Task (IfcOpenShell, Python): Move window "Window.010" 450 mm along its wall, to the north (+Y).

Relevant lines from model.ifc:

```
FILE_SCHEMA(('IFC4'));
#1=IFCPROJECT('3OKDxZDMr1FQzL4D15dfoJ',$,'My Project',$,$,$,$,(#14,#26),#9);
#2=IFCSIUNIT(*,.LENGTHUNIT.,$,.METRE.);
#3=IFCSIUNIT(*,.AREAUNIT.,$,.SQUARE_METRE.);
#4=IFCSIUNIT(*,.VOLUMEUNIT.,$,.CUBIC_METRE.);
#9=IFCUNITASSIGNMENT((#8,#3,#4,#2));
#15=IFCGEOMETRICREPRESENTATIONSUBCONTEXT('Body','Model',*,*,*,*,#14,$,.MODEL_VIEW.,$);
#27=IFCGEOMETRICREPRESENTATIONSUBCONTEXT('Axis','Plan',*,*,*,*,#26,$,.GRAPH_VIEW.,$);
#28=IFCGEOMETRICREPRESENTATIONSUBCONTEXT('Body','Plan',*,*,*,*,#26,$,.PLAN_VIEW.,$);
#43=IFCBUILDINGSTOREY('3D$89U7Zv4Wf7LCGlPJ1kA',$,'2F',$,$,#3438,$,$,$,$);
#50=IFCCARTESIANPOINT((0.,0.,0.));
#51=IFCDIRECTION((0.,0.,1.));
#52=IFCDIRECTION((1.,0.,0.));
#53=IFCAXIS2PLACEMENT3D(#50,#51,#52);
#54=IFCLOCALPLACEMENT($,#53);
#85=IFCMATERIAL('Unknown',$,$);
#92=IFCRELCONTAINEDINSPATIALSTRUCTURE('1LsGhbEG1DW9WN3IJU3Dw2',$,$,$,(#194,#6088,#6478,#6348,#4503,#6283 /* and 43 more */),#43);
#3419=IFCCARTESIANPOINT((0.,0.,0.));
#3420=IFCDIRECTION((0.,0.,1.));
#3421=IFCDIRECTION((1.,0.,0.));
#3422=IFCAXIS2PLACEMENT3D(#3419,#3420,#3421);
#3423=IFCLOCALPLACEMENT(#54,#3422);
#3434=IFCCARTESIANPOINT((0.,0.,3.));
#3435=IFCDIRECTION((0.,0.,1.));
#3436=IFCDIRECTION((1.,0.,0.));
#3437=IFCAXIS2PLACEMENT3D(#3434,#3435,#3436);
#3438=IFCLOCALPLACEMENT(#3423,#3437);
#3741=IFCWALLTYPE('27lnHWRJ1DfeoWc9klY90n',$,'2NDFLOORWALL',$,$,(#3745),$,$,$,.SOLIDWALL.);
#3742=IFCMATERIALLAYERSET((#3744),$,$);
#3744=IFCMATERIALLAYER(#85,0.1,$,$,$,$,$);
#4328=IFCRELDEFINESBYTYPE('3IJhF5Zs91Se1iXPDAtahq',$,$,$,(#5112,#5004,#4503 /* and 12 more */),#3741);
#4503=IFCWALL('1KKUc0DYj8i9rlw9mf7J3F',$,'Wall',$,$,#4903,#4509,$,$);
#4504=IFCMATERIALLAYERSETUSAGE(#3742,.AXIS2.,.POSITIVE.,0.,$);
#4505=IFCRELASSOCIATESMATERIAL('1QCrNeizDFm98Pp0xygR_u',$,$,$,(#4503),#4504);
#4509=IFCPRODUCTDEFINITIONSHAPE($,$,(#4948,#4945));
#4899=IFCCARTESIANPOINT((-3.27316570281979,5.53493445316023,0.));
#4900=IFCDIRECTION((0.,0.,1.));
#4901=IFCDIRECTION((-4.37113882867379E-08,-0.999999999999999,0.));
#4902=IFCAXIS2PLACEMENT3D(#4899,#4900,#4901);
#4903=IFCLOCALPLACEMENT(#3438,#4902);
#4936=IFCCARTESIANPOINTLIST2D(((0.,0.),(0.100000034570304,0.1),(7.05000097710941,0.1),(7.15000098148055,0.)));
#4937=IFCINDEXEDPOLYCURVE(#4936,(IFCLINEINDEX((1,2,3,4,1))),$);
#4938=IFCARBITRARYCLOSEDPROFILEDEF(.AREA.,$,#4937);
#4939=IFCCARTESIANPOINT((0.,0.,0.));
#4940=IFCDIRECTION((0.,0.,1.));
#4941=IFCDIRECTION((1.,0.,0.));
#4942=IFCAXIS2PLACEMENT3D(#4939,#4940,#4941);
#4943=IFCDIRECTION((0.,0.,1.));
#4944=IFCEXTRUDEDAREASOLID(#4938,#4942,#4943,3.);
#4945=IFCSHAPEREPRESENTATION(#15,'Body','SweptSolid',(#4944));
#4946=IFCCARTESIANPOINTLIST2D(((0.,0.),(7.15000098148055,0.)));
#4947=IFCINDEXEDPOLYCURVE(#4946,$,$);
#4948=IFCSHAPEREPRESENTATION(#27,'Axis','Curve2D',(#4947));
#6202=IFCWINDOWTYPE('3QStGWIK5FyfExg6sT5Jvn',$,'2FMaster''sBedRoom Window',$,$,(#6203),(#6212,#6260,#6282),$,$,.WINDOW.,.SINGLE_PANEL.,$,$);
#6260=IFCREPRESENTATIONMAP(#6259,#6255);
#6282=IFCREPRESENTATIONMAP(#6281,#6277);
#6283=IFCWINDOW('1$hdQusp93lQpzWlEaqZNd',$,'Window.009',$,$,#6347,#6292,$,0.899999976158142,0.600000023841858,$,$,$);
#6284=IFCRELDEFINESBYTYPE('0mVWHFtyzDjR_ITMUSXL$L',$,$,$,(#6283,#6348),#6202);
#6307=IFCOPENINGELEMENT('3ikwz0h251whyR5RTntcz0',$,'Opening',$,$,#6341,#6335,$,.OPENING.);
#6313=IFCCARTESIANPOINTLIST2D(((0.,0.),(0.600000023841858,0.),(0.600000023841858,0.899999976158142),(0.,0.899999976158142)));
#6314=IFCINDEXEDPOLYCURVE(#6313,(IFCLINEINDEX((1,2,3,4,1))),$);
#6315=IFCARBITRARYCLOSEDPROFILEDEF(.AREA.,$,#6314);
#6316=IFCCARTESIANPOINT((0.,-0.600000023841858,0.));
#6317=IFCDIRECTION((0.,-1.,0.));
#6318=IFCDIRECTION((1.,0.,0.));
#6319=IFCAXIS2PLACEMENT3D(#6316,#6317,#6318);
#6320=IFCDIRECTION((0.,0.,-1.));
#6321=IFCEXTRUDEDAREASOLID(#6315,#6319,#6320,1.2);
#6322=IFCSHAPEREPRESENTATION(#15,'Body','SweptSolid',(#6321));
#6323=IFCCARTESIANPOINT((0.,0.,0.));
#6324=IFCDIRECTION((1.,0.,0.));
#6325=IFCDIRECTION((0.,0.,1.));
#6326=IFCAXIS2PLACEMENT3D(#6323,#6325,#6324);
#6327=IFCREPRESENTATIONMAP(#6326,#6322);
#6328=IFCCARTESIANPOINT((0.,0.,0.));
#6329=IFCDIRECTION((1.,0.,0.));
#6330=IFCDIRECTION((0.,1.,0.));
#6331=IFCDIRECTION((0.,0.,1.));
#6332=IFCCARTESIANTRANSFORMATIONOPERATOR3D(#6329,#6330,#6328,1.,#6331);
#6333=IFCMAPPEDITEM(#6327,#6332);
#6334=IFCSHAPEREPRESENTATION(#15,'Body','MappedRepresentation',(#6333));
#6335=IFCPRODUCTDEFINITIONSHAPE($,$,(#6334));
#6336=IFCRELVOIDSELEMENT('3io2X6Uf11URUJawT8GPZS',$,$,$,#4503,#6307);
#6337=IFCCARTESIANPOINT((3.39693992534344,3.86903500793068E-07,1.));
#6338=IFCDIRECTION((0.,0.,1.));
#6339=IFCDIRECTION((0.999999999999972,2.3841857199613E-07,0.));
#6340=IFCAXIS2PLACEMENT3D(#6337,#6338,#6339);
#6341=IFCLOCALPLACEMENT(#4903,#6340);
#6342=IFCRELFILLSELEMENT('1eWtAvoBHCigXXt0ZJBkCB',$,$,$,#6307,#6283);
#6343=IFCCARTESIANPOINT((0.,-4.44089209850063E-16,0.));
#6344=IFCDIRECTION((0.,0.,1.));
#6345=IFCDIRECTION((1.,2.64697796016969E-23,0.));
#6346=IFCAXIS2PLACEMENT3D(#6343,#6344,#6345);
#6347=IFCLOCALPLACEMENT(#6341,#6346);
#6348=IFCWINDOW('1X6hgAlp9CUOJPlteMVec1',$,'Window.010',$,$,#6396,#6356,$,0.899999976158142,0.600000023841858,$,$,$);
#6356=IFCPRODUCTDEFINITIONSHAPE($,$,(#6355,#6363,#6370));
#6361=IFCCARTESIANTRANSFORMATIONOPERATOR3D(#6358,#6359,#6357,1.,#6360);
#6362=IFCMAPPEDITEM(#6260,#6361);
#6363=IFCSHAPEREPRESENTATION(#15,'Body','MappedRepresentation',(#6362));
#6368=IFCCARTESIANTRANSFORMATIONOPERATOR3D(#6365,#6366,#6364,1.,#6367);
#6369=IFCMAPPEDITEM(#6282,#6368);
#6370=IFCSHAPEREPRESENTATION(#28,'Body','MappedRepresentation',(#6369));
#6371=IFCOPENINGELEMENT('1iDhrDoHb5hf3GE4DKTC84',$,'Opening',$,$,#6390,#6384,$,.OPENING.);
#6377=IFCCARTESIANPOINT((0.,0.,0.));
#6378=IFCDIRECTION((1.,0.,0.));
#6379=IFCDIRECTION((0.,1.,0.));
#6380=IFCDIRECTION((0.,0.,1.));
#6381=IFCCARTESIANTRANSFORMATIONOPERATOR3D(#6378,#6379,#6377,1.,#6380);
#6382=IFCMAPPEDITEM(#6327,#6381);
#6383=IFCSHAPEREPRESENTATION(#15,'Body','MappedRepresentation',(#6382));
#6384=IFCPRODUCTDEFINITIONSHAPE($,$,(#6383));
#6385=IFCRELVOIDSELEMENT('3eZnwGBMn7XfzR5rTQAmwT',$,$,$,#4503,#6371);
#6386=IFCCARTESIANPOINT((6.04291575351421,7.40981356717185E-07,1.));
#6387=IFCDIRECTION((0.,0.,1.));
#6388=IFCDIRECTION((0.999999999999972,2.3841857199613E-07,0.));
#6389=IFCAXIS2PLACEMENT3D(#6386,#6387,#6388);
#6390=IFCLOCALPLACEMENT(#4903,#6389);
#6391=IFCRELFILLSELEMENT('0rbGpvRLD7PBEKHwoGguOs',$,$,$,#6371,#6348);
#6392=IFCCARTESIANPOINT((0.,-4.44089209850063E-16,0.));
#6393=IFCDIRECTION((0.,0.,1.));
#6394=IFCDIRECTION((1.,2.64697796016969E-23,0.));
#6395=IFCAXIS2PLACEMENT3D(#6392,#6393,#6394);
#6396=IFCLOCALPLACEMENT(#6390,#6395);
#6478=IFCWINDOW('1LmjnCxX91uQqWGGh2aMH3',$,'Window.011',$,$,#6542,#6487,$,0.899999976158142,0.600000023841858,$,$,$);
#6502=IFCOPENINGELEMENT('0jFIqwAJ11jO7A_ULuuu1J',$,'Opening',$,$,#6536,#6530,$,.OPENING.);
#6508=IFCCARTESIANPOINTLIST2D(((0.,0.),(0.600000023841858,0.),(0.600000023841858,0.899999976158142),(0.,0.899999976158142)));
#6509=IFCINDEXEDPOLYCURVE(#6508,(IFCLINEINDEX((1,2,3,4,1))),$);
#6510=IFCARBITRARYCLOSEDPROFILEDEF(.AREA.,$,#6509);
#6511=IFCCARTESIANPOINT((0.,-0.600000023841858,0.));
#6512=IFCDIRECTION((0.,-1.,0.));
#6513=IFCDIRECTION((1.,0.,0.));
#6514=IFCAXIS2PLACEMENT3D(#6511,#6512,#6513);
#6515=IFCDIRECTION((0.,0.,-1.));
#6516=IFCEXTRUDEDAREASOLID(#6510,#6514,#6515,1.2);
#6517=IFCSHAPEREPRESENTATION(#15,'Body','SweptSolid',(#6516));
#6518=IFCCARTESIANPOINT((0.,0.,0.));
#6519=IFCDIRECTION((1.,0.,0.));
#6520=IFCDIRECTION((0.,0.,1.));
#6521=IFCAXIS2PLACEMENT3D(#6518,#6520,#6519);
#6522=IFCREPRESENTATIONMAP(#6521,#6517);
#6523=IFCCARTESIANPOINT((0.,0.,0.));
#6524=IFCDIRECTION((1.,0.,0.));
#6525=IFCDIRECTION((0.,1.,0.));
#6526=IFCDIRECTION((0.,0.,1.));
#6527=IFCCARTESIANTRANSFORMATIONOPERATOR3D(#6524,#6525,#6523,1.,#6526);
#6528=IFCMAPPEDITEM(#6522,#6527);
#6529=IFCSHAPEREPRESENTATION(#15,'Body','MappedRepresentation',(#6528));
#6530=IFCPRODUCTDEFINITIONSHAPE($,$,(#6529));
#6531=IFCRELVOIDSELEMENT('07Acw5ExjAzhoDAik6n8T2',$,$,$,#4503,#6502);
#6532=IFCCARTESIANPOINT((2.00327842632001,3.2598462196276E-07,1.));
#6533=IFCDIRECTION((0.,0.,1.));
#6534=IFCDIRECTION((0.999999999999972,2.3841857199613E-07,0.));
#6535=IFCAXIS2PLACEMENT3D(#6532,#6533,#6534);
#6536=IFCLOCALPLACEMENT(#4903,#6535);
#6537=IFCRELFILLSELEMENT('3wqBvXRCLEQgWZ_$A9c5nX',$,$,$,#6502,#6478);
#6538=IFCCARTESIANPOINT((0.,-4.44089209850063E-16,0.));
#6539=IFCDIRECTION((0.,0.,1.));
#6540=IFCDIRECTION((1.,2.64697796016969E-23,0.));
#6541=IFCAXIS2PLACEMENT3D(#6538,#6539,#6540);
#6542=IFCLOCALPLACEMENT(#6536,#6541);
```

```python
import ifcopenshell
import ifcopenshell.api.geometry
import ifcopenshell.util.placement
import ifcopenshell.util.unit

model = ifcopenshell.open("model.ifc")
unit_scale = ifcopenshell.util.unit.calculate_unit_scale(model)

window = model.by_guid("1X6hgAlp9CUOJPlteMVec1")
opening = window.FillsVoids[0].RelatingOpeningElement
wall = opening.VoidsElements[0].RelatingBuildingElement

wall_matrix = ifcopenshell.util.placement.get_local_placement(wall.ObjectPlacement)
shift = wall_matrix[:3, 0] * -0.45 / unit_scale
before = ifcopenshell.util.placement.get_local_placement(window.ObjectPlacement)[:3, 3].copy()

# The window is placed relative to its opening, so it follows when the opening moves.
matrix = ifcopenshell.util.placement.get_local_placement(opening.ObjectPlacement)
matrix[:3, 3] += shift
ifcopenshell.api.geometry.edit_object_placement(
    model, product=opening, matrix=matrix, is_si=False, should_transform_children=True
)

after = ifcopenshell.util.placement.get_local_placement(window.ObjectPlacement)[:3, 3]
print("window moved by", (after - before).round(3) + 0.0)

model.write("model_v2.ifc")
```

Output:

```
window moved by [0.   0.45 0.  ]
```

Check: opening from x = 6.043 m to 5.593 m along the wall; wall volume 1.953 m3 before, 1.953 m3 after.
